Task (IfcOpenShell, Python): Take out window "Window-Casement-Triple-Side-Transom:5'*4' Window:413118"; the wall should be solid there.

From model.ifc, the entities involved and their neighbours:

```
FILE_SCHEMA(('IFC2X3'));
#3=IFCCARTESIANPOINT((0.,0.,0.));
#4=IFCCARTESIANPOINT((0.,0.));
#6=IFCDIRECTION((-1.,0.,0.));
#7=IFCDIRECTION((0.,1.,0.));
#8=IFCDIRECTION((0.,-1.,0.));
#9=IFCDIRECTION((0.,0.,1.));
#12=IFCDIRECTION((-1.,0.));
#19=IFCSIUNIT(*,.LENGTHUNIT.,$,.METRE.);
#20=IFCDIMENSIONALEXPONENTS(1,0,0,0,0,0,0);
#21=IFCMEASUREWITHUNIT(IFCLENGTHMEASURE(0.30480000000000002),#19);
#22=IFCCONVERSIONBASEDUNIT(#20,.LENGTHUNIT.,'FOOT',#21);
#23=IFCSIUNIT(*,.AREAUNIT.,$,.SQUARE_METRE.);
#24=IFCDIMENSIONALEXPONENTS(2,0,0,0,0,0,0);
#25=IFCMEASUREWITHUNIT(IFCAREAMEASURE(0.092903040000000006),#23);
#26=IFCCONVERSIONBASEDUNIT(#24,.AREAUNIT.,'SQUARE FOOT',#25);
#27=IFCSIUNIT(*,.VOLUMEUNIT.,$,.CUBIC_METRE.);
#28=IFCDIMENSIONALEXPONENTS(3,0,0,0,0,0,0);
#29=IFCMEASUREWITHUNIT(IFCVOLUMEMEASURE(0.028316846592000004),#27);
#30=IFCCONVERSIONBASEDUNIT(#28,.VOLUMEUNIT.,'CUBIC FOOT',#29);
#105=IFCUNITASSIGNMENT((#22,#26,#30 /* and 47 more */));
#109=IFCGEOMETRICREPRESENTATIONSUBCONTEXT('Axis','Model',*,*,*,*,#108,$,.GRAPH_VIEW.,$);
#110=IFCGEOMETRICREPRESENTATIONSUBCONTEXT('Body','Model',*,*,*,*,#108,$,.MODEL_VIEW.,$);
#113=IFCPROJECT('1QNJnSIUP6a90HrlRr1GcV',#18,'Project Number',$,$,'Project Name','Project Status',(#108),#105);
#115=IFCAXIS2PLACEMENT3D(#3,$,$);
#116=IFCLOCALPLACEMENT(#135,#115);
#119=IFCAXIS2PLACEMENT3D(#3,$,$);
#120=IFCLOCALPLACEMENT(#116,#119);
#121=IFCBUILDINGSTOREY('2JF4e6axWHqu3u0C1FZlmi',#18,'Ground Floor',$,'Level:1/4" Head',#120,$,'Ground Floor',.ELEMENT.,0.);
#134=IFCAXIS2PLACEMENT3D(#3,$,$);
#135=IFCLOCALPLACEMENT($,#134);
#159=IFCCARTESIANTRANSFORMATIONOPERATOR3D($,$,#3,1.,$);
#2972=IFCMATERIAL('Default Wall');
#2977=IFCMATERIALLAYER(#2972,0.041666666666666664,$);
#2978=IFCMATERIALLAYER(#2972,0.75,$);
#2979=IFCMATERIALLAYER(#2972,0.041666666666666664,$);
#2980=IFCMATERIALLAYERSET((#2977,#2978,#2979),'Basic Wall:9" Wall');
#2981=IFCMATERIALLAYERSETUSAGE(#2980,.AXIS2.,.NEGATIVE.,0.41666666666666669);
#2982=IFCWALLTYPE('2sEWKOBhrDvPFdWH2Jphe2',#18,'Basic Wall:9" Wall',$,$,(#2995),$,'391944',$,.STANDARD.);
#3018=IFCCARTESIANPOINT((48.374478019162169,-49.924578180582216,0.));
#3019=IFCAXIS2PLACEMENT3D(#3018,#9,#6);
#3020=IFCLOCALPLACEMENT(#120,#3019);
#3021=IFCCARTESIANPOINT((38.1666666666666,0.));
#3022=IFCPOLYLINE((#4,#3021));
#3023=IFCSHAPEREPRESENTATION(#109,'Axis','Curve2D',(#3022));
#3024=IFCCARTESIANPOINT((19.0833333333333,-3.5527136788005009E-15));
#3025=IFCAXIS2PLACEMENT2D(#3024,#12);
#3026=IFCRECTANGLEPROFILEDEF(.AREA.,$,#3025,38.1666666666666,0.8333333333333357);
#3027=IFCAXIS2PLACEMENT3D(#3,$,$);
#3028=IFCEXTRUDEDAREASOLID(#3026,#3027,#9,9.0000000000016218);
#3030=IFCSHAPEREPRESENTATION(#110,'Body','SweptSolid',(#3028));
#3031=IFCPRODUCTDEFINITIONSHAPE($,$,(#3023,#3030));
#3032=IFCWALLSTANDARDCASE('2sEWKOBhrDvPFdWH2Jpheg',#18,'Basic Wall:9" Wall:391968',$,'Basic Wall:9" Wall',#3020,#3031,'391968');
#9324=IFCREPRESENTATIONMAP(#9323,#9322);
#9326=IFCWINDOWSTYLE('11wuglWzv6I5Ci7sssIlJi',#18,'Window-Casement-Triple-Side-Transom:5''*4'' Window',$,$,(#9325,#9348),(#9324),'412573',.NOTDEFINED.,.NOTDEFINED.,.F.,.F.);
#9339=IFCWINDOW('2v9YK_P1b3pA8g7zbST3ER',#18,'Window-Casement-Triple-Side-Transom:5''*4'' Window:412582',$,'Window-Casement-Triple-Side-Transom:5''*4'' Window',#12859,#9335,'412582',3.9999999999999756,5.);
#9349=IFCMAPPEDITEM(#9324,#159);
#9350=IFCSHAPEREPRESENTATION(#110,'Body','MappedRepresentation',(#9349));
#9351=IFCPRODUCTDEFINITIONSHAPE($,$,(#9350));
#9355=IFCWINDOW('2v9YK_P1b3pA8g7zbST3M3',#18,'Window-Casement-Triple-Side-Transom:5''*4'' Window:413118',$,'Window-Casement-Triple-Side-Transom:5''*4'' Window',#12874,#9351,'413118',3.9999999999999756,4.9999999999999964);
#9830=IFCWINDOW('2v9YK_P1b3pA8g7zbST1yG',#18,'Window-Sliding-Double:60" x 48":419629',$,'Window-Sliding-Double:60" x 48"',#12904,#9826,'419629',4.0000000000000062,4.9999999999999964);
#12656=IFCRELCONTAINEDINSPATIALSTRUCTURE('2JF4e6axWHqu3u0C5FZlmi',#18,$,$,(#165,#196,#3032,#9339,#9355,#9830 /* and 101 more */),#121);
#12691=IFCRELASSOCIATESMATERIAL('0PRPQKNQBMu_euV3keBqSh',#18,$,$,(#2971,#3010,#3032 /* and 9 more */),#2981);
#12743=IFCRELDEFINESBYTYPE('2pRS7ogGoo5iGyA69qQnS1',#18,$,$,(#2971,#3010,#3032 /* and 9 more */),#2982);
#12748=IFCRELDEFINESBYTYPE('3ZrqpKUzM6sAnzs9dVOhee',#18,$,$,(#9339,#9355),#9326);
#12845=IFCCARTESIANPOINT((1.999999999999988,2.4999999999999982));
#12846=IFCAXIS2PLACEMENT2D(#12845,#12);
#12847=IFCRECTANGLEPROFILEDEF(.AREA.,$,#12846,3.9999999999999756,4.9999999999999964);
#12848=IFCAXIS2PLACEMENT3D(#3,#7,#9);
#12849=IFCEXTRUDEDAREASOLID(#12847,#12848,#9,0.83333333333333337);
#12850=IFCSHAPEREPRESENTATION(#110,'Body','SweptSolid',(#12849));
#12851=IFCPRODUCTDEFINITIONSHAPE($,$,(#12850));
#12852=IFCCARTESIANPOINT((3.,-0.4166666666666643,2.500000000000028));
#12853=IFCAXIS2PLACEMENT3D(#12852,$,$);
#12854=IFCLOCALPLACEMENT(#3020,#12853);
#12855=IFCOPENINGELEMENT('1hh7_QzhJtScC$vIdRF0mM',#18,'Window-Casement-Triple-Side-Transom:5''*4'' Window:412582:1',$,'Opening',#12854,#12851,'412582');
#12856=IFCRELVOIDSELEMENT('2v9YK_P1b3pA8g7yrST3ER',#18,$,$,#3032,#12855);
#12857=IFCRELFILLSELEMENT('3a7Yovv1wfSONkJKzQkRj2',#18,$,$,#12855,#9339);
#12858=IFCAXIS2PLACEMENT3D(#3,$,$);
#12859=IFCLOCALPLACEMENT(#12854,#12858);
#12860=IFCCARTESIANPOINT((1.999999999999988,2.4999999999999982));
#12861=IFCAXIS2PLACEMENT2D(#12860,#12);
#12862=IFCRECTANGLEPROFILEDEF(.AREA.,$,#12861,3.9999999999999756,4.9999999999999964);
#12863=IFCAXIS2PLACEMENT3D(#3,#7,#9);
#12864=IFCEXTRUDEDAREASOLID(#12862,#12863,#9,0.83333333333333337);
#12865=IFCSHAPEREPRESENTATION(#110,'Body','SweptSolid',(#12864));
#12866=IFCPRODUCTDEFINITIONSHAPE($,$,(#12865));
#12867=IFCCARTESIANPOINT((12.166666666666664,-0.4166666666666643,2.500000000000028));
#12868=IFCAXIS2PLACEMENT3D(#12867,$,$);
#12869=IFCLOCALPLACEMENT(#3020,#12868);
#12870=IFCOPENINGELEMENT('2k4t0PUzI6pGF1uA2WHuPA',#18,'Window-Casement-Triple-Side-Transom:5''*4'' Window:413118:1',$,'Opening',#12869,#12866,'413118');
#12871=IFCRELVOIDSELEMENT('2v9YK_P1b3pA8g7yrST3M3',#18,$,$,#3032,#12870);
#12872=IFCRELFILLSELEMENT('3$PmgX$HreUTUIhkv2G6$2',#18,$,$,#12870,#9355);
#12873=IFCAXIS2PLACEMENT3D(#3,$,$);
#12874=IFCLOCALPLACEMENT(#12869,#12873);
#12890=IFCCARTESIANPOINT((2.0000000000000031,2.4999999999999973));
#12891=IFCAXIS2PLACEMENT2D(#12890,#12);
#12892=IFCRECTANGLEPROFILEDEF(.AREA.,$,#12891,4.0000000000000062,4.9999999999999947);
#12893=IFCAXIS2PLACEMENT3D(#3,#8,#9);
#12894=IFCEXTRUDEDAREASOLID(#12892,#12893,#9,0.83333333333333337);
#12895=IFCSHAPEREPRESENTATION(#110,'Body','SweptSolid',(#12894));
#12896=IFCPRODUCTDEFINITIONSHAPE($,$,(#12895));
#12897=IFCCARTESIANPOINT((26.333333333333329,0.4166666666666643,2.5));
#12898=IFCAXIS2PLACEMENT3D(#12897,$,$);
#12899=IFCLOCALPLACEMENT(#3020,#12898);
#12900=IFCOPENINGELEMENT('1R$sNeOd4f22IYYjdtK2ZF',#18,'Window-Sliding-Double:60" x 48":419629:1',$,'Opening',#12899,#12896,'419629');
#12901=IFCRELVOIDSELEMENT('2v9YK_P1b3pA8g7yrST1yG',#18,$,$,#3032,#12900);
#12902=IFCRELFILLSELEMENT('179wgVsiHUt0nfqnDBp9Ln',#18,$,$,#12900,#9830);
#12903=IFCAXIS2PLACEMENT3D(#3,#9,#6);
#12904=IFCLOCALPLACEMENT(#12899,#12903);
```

```python
import ifcopenshell
import ifcopenshell.api.feature
import ifcopenshell.api.root
import ifcopenshell.geom
import ifcopenshell.util.shape

model = ifcopenshell.open("model.ifc")
settings = ifcopenshell.geom.settings()


def volume(element):
    """Net volume in cubic metres, openings subtracted."""
    shape = ifcopenshell.geom.create_shape(settings, element)
    return ifcopenshell.util.shape.get_volume(shape.geometry)


window = model.by_id(9355)
opening = window.FillsVoids[0].RelatingOpeningElement
wall = opening.VoidsElements[0].RelatingBuildingElement
before = volume(wall)

ifcopenshell.api.root.remove_product(model, product=window)
ifcopenshell.api.feature.remove_feature(model, feature=opening)

after = volume(wall)

print(f"wall volume {before:.3f} -> {after:.3f} m3")

model.write("model_edited.ifc")
```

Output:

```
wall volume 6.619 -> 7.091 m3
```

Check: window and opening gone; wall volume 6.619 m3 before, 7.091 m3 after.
